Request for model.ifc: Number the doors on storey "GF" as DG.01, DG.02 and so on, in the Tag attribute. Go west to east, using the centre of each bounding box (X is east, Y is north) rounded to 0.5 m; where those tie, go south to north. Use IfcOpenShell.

First a look at what the model holds.

```python
import ifcopenshell
import ifcopenshell.util.element
import ifcopenshell.util.placement

model = ifcopenshell.open("model.ifc")
print(model.schema)
storey = next(s for s in model.by_type("IfcBuildingStorey") if s.Name == "GF")
doors = [e for e in ifcopenshell.util.element.get_decomposition(storey) if e.is_a("IfcDoor")]
for e in sorted(doors, key=lambda e: e.id()):
    origin = ifcopenshell.util.placement.get_local_placement(e.ObjectPlacement)[:3, 3]
    print(e.id(), e.Tag, e.Name, origin.round(2) + 0.0, sep=" | ")
```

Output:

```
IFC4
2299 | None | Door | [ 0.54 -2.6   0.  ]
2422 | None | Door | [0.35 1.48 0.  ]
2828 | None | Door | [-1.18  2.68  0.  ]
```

```python
import ifcopenshell
import ifcopenshell.geom
import ifcopenshell.util.element
import ifcopenshell.util.shape

model = ifcopenshell.open("model.ifc")
settings = ifcopenshell.geom.settings()
settings.set("use-world-coords", True)


def centre(element):
    shape = ifcopenshell.geom.create_shape(settings, element)
    return ifcopenshell.util.shape.get_bbox_centroid(shape.geometry)


storey = next(s for s in model.by_type("IfcBuildingStorey") if s.Name == "GF")
doors = [e for e in ifcopenshell.util.element.get_decomposition(storey) if e.is_a("IfcDoor")]

# Insertion points can sit at a corner or the storey origin, so sort by the geometry (in metres).
centres = {e: centre(e) for e in doors}
doors.sort(key=lambda e: (round(centres[e][0] / 0.5), centres[e][1]))

for i, e in enumerate(doors, start=1):
    number = f"DG.{i:02d}"
    e.Tag = number
    print(e.id(), number)

model.write("model_rev.ifc")
```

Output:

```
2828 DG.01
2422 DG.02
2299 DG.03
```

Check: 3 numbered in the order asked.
